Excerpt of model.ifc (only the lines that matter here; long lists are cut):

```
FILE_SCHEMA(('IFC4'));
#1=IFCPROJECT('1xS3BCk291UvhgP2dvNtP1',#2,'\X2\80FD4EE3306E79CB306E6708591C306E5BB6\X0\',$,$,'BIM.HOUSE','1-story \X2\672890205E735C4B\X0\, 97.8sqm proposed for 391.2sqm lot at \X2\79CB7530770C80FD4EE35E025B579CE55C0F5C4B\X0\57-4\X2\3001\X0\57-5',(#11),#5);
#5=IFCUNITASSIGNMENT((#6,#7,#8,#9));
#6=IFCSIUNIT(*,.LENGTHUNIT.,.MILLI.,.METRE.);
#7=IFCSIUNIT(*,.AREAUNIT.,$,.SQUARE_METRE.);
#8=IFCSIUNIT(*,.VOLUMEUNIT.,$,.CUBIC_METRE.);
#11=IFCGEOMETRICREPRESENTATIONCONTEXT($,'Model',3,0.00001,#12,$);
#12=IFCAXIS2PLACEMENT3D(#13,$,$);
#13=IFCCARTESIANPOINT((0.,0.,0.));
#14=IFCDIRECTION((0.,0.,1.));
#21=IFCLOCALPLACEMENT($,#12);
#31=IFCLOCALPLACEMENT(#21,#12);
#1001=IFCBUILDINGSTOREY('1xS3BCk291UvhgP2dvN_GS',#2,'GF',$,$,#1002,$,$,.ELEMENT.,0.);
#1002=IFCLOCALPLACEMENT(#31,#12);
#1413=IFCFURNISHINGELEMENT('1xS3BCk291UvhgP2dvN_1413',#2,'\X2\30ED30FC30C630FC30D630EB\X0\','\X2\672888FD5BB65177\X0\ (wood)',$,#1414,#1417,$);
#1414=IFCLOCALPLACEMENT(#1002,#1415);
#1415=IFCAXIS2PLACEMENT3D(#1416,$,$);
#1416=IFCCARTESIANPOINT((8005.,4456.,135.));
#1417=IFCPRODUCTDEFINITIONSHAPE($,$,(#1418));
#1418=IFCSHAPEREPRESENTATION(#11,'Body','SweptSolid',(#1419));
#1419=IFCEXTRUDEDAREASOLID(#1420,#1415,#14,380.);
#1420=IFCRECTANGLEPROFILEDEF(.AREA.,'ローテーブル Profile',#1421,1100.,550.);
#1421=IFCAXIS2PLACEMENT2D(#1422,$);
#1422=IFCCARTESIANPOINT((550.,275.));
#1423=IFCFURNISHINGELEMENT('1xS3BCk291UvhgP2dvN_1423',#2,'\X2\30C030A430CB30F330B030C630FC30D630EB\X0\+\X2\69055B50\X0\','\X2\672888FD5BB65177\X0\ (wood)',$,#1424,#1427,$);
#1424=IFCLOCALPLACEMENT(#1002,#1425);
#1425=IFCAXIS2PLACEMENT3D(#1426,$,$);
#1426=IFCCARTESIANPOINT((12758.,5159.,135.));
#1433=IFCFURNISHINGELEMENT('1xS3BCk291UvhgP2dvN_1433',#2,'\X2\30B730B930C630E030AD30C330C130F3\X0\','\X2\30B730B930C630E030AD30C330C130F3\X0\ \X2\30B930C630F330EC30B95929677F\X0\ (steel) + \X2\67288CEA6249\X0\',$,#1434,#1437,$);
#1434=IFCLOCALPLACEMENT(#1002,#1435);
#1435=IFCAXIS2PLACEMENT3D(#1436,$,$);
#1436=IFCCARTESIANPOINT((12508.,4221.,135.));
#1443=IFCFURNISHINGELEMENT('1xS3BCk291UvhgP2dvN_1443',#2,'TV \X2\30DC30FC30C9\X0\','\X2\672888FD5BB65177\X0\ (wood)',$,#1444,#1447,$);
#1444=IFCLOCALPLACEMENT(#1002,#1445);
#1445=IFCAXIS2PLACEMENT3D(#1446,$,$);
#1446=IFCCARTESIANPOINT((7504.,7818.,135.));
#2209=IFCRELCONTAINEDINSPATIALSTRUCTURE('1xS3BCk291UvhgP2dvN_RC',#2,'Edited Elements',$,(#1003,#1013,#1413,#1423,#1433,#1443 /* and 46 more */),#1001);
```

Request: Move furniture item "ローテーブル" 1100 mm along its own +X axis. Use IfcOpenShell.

```python
import ifcopenshell
import ifcopenshell.api.geometry
import ifcopenshell.util.placement

model = ifcopenshell.open("model.ifc")

item = model.by_guid("1xS3BCk291UvhgP2dvN_1413")
matrix = ifcopenshell.util.placement.get_local_placement(item.ObjectPlacement)
matrix[:3, 3] += matrix[:3, 0] * 1100.0
ifcopenshell.api.geometry.edit_object_placement(model, product=item, matrix=matrix, is_si=False)

print(ifcopenshell.util.placement.get_local_placement(item.ObjectPlacement).round(3) + 0.0)

model.write("model-out.ifc")
```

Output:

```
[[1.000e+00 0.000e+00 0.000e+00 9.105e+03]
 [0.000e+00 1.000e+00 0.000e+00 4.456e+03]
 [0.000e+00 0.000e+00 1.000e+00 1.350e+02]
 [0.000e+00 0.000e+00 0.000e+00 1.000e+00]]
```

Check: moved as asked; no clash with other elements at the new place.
